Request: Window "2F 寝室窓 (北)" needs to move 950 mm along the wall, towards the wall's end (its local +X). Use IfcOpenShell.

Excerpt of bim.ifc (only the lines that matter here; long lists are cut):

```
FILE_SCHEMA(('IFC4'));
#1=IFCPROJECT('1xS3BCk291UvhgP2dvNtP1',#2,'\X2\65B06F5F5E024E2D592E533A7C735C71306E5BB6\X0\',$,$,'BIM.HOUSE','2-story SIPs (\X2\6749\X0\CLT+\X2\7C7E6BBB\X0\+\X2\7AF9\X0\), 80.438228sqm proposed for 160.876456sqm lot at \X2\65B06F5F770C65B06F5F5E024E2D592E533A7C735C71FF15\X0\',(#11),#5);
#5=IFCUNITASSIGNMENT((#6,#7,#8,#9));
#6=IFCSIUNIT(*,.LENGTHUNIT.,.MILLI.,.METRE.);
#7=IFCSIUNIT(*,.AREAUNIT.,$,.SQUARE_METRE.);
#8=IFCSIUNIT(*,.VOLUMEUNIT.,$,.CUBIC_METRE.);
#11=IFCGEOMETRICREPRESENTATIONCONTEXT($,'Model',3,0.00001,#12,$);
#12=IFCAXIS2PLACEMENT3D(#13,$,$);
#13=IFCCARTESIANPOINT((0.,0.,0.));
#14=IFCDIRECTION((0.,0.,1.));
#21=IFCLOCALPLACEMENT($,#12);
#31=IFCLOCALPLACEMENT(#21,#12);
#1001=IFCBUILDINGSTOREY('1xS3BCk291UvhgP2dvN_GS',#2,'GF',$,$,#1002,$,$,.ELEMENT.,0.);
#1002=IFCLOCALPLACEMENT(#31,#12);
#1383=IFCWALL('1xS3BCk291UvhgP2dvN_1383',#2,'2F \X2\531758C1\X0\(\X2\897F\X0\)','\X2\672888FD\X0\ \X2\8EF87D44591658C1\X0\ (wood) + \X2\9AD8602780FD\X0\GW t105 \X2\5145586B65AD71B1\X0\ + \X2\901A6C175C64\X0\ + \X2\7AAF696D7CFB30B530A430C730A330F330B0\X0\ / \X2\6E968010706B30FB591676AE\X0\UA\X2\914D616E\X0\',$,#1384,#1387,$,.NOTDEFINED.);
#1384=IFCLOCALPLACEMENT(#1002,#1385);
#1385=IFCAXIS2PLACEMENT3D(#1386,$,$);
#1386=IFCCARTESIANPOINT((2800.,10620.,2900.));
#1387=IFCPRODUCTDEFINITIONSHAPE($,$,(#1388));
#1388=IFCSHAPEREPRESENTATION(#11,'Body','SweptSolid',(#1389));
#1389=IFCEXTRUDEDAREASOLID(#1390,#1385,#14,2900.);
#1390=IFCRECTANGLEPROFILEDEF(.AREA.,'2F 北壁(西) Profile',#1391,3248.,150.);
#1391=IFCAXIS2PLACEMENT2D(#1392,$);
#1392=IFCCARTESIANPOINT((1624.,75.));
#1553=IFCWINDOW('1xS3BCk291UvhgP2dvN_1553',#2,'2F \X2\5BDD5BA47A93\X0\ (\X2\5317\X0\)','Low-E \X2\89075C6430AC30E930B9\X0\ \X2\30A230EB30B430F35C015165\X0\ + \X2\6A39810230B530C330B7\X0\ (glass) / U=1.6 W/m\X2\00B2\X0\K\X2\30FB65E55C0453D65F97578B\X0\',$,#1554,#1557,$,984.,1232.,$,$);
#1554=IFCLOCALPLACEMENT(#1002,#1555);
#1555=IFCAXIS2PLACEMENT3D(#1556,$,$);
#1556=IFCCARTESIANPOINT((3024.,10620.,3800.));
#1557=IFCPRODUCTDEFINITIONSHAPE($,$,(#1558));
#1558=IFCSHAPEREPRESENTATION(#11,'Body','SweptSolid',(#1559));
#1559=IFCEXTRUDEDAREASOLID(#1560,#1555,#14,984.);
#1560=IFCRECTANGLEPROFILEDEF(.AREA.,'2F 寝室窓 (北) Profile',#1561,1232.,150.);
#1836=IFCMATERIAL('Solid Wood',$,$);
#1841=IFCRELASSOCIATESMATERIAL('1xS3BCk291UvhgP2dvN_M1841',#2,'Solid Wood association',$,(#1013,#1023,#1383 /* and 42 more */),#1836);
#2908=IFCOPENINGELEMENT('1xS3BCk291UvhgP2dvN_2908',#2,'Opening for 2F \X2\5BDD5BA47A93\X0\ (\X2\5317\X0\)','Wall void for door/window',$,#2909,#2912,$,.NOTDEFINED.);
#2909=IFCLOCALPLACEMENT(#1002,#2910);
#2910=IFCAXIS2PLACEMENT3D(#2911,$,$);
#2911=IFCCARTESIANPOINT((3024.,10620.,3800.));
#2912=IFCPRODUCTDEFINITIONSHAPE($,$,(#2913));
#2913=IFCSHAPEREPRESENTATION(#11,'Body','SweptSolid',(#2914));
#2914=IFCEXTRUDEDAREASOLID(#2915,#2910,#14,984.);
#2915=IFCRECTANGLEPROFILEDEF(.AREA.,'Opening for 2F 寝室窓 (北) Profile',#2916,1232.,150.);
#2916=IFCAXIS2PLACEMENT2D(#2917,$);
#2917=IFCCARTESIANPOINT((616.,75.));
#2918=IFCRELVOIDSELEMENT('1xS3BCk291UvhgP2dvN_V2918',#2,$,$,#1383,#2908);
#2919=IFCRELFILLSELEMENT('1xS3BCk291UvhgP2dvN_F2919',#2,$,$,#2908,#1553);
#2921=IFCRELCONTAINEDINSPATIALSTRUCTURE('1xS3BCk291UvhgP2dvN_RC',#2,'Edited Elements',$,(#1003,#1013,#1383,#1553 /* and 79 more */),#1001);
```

```python
import ifcopenshell
import ifcopenshell.api.geometry
import ifcopenshell.util.placement
import ifcopenshell.util.unit

model = ifcopenshell.open("bim.ifc")
unit_scale = ifcopenshell.util.unit.calculate_unit_scale(model)

window = model.by_guid("1xS3BCk291UvhgP2dvN_1553")
opening = window.FillsVoids[0].RelatingOpeningElement
wall = opening.VoidsElements[0].RelatingBuildingElement

wall_matrix = ifcopenshell.util.placement.get_local_placement(wall.ObjectPlacement)
shift = wall_matrix[:3, 0] * 0.95 / unit_scale
before = ifcopenshell.util.placement.get_local_placement(window.ObjectPlacement)[:3, 3].copy()

# The window is not placed relative to its opening, so move both.
for product in (opening, window):
    matrix = ifcopenshell.util.placement.get_local_placement(product.ObjectPlacement)
    matrix[:3, 3] += shift
    ifcopenshell.api.geometry.edit_object_placement(model, product=product, matrix=matrix, is_si=False)

after = ifcopenshell.util.placement.get_local_placement(window.ObjectPlacement)[:3, 3]
print("window moved by", (after - before).round(3) + 0.0)

model.write("bim_updated.ifc")
```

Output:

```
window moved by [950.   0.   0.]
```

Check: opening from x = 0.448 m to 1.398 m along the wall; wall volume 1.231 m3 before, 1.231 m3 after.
